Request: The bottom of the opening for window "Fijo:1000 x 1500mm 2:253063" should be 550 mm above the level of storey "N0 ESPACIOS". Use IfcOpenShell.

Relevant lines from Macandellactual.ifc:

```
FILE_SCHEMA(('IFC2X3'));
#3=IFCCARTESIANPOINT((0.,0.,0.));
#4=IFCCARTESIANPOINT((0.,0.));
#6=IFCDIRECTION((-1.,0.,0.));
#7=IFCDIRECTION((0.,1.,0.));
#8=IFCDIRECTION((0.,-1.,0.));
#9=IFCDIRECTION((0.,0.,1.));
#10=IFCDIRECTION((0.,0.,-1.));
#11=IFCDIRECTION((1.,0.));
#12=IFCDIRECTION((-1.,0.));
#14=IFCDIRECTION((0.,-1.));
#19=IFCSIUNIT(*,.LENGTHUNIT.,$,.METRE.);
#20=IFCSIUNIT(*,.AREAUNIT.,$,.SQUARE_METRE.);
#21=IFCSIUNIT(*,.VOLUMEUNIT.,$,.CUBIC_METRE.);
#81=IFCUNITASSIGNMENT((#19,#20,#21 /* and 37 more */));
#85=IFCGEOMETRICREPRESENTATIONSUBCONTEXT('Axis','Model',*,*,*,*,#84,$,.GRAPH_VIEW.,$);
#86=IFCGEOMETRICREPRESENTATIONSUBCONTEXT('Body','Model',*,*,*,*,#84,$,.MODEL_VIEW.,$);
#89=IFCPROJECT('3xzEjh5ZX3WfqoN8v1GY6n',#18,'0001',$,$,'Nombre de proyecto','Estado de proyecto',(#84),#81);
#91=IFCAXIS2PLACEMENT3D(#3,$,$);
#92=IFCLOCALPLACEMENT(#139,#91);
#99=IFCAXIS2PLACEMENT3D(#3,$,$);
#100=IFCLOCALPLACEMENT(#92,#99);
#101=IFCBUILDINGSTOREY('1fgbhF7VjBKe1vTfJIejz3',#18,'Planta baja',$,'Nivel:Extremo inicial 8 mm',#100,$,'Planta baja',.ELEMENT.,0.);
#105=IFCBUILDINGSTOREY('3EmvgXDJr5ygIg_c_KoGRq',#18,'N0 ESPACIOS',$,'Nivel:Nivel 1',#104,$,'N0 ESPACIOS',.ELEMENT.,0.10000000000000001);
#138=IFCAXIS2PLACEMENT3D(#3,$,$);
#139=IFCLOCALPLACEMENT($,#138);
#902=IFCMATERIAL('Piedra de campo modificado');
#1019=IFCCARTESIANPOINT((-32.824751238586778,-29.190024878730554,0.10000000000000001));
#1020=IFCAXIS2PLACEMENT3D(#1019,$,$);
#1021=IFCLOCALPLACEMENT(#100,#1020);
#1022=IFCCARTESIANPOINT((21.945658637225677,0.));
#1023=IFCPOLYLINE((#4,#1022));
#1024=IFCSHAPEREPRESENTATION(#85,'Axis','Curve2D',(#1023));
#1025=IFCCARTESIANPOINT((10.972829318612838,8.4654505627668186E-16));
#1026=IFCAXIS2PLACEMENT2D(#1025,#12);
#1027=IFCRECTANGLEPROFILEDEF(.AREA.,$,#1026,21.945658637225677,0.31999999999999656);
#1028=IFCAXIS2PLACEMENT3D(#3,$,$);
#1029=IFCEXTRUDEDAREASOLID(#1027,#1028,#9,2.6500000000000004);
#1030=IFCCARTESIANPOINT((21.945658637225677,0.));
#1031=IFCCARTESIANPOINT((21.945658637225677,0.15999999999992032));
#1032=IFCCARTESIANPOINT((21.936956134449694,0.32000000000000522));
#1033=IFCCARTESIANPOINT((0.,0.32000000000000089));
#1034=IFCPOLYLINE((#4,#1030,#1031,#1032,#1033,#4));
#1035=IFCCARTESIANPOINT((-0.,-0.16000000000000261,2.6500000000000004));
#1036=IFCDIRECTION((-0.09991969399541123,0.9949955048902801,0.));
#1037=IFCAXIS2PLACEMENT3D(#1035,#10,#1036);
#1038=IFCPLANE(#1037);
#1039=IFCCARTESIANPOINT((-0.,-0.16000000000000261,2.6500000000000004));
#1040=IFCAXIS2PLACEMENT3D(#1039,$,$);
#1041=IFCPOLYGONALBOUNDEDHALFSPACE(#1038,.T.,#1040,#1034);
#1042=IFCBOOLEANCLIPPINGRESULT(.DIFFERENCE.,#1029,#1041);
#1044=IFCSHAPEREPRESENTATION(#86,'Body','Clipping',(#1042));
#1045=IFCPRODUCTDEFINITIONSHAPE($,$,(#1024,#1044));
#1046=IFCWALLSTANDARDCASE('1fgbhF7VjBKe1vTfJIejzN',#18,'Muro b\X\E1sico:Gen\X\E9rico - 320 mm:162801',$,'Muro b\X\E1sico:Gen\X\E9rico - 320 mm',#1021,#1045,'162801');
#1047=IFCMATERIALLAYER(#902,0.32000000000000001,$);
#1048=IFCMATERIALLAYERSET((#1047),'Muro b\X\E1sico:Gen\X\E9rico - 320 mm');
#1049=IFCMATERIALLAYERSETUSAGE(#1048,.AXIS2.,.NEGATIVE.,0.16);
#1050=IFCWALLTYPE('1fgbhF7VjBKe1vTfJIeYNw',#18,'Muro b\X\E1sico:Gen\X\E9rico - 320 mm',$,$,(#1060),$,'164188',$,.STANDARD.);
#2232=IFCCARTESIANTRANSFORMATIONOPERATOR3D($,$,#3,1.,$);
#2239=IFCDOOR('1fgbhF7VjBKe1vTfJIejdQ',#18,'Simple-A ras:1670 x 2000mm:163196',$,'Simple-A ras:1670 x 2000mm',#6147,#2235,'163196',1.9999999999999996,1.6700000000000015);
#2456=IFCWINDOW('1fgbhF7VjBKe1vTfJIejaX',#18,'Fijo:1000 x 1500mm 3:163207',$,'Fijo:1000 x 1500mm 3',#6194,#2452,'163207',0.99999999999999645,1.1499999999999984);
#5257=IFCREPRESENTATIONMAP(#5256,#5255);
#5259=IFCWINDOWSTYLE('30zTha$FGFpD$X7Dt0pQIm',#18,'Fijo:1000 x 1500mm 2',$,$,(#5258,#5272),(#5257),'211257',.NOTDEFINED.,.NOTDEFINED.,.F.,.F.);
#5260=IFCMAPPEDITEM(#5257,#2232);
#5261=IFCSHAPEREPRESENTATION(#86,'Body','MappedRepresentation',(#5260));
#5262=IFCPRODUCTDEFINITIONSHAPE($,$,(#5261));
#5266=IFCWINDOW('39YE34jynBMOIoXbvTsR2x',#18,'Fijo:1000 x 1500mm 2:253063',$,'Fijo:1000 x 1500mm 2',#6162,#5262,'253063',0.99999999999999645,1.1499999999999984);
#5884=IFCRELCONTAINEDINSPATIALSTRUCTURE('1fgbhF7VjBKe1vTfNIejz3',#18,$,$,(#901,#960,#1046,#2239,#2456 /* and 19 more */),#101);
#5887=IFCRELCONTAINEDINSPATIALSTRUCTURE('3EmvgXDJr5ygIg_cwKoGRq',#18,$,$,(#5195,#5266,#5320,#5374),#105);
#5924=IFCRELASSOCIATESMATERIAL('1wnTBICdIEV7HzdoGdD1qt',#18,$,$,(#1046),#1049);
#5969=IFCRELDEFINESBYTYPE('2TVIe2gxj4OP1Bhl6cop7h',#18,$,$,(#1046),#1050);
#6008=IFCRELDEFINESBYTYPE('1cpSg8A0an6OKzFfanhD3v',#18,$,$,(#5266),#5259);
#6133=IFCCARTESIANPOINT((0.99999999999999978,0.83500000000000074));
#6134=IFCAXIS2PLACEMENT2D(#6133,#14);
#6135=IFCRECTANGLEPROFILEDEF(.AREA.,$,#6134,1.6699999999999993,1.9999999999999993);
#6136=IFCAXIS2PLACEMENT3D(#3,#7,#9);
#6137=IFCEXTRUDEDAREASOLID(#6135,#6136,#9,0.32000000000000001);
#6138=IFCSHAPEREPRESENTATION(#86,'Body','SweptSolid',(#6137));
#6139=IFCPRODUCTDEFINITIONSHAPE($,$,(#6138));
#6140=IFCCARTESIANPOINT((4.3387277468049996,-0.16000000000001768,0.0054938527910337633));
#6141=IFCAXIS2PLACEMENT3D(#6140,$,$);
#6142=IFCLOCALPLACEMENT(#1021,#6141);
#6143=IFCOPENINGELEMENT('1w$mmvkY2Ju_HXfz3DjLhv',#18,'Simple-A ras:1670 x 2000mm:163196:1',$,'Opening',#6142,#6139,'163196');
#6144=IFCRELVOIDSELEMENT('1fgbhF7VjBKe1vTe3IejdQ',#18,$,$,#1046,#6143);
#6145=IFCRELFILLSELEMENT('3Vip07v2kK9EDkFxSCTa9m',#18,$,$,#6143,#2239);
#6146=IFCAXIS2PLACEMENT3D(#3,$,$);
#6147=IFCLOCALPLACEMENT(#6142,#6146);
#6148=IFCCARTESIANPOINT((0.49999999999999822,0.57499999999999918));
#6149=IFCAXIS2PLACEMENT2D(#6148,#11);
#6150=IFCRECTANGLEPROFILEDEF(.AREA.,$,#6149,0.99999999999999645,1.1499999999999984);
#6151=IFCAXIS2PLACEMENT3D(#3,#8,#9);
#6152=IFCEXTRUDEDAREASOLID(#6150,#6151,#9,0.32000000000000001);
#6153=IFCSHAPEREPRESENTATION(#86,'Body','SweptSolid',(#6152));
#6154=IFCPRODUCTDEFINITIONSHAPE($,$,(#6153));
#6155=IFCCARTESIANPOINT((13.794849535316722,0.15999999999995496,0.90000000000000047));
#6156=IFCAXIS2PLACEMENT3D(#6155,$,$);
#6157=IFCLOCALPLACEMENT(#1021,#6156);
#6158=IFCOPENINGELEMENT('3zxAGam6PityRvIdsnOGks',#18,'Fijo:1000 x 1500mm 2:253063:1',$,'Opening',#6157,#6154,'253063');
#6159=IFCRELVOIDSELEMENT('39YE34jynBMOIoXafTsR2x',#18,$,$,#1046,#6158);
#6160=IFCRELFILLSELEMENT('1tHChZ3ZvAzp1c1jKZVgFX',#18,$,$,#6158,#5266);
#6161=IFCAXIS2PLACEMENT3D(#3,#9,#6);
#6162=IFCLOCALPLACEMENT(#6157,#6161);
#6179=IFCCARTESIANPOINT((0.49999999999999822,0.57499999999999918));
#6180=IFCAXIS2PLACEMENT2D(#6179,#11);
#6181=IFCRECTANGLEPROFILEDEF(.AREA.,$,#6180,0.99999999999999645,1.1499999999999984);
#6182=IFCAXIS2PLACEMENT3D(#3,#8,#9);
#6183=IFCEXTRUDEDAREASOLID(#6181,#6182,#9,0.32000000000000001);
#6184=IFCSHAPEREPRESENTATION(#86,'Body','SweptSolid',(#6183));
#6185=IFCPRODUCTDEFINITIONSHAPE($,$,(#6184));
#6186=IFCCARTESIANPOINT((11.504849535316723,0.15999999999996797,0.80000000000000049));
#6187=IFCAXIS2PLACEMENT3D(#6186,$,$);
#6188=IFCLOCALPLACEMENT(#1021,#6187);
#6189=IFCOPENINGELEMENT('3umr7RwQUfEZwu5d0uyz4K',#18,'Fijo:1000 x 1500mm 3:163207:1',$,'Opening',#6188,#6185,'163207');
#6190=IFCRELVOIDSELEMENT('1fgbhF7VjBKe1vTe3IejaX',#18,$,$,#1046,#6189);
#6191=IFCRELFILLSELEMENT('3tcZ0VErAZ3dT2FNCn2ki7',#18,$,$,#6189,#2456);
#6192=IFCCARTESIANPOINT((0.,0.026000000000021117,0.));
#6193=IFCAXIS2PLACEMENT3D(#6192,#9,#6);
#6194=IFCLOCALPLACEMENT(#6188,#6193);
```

```python
import numpy as np
import ifcopenshell
import ifcopenshell.api.geometry
import ifcopenshell.geom
import ifcopenshell.util.element
import ifcopenshell.util.placement
import ifcopenshell.util.shape
import ifcopenshell.util.unit

model = ifcopenshell.open("Macandellactual.ifc")
unit_scale = ifcopenshell.util.unit.calculate_unit_scale(model)

window = model.by_guid("39YE34jynBMOIoXbvTsR2x")
opening = window.FillsVoids[0].RelatingOpeningElement
storey = ifcopenshell.util.element.get_container(window, ifc_class="IfcBuildingStorey")
level = ifcopenshell.util.placement.get_local_placement(storey.ObjectPlacement)[2, 3]

# The opening's origin need not be at the sill, so measure its lowest point.
shape = ifcopenshell.geom.create_shape(ifcopenshell.geom.settings(), opening)
bottom = ifcopenshell.util.shape.get_shape_bottom_elevation(shape, shape.geometry) / unit_scale
dz = level + 0.55 / unit_scale - bottom

shift = np.array([0.0, 0.0, dz])
# The window is placed relative to its opening, so it follows when the opening moves.
matrix = ifcopenshell.util.placement.get_local_placement(opening.ObjectPlacement)
matrix[:3, 3] += shift
ifcopenshell.api.geometry.edit_object_placement(
    model, product=opening, matrix=matrix, is_si=False, should_transform_children=True
)

print(f"moved by {dz * unit_scale:+.3f} m")

model.write("Macandellactual_edited.ifc")
```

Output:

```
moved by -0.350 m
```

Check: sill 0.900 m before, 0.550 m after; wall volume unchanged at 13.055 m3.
